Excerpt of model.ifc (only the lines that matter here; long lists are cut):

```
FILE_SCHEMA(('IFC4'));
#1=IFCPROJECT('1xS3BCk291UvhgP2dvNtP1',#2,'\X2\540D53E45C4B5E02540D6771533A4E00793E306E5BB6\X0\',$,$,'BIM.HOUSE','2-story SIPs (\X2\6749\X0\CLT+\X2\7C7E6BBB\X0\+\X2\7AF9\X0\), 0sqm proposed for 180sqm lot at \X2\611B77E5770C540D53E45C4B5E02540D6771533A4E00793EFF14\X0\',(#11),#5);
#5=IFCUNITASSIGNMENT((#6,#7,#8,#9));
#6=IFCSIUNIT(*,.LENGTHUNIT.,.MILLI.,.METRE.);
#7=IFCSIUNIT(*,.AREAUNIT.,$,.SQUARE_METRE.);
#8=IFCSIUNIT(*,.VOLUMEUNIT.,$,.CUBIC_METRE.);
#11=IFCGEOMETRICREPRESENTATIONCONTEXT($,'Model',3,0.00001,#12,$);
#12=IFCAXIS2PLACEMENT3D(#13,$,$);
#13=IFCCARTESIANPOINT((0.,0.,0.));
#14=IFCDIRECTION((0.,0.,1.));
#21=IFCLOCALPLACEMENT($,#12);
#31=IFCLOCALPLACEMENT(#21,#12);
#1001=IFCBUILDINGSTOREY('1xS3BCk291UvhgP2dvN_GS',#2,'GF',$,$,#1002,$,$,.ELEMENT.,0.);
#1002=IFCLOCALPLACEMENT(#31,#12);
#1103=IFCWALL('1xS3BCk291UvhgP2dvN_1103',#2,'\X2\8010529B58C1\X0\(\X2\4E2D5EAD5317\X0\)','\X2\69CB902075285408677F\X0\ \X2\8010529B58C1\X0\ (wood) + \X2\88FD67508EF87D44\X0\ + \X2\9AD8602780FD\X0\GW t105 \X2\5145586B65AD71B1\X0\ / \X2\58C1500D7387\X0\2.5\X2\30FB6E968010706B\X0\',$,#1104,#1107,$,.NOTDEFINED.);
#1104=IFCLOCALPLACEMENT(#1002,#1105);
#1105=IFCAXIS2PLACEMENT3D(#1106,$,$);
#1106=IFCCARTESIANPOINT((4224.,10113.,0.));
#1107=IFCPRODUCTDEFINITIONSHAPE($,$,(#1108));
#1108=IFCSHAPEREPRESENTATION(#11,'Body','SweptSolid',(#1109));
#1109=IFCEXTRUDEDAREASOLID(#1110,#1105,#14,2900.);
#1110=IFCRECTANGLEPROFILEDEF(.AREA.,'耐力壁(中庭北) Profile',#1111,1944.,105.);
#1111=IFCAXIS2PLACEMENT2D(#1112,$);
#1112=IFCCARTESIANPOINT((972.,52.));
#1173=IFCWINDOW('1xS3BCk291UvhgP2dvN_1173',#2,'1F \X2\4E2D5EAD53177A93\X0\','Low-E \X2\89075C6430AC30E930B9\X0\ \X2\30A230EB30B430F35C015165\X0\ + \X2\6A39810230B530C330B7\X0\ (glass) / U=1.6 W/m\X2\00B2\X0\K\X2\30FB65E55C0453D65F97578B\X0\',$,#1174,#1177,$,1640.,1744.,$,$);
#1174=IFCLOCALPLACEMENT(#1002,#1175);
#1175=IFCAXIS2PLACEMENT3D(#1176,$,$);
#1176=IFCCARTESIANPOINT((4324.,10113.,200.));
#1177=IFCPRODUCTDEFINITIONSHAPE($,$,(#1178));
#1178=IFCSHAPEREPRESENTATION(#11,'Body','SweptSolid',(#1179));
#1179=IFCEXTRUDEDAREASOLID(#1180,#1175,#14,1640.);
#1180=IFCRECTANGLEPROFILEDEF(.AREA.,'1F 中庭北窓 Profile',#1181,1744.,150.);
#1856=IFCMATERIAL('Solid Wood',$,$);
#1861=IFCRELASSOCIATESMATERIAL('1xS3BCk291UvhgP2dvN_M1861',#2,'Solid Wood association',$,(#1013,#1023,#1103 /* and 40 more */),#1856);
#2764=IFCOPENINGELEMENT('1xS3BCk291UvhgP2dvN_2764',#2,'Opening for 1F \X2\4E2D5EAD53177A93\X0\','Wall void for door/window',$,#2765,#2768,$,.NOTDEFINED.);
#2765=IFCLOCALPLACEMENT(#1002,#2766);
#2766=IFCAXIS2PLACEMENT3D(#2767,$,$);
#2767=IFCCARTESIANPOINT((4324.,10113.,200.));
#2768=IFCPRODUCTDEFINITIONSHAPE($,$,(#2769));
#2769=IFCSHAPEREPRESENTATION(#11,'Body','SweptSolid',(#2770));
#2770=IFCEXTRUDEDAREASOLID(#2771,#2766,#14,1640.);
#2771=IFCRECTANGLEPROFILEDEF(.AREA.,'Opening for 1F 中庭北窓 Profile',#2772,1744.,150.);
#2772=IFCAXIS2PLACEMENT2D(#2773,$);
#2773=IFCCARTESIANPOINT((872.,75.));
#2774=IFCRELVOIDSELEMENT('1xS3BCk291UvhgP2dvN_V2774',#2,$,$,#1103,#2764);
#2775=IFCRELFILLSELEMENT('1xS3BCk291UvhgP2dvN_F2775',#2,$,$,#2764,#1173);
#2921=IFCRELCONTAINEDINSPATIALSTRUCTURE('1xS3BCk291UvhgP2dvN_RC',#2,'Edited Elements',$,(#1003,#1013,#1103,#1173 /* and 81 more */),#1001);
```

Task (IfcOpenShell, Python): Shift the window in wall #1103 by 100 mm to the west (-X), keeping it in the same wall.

```python
import ifcopenshell
import ifcopenshell.api.geometry
import ifcopenshell.util.placement

model = ifcopenshell.open("model.ifc")

window = model.by_id(1173)
opening = window.FillsVoids[0].RelatingOpeningElement
wall = opening.VoidsElements[0].RelatingBuildingElement

wall_matrix = ifcopenshell.util.placement.get_local_placement(wall.ObjectPlacement)
shift = wall_matrix[:3, 0] * -100.0
before = ifcopenshell.util.placement.get_local_placement(window.ObjectPlacement)[:3, 3].copy()

# The window is not placed relative to its opening, so move both.
for product in (opening, window):
    matrix = ifcopenshell.util.placement.get_local_placement(product.ObjectPlacement)
    matrix[:3, 3] += shift
    ifcopenshell.api.geometry.edit_object_placement(model, product=product, matrix=matrix, is_si=False)

after = ifcopenshell.util.placement.get_local_placement(window.ObjectPlacement)[:3, 3]
print("window moved by", (after - before).round(3) + 0.0)

model.write("model-out.ifc")
```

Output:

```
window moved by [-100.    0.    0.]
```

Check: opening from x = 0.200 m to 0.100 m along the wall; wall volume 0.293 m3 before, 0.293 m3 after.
